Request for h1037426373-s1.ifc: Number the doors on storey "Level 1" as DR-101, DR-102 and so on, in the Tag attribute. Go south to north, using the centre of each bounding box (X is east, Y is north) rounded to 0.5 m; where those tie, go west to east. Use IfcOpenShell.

First a look at what the model holds.

```python
import ifcopenshell
import ifcopenshell.util.element
import ifcopenshell.util.placement

model = ifcopenshell.open("h1037426373-s1.ifc")
print(model.schema)
storey = next(s for s in model.by_type("IfcBuildingStorey") if s.Name == "Level 1")
doors = [e for e in ifcopenshell.util.element.get_decomposition(storey) if e.is_a("IfcDoor")]
for e in sorted(doors, key=lambda e: e.id()):
    origin = ifcopenshell.util.placement.get_local_placement(e.ObjectPlacement)[:3, 3]
    print(e.id(), e.Tag, e.Name, origin.round(2) + 0.0, sep=" | ")
```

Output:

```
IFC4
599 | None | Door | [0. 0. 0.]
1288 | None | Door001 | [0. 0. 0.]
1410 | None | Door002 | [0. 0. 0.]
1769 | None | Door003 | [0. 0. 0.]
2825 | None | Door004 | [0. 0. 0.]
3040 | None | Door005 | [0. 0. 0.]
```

```python
import ifcopenshell
import ifcopenshell.geom
import ifcopenshell.util.element
import ifcopenshell.util.shape

model = ifcopenshell.open("h1037426373-s1.ifc")
settings = ifcopenshell.geom.settings()
settings.set("use-world-coords", True)


def centre(element):
    shape = ifcopenshell.geom.create_shape(settings, element)
    return ifcopenshell.util.shape.get_bbox_centroid(shape.geometry)


storey = next(s for s in model.by_type("IfcBuildingStorey") if s.Name == "Level 1")
doors = [e for e in ifcopenshell.util.element.get_decomposition(storey) if e.is_a("IfcDoor")]

# Insertion points can sit at a corner or the storey origin, so sort by the geometry (in metres).
centres = {e: centre(e) for e in doors}
doors.sort(key=lambda e: (round(centres[e][1] / 0.5), centres[e][0]))

for i, e in enumerate(doors, start=1):
    number = f"DR-1{i:02d}"
    e.Tag = number
    print(e.id(), number)

model.write("h1037426373-s1_updated.ifc")
```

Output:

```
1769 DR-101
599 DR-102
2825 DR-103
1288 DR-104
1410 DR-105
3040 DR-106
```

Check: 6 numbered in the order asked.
